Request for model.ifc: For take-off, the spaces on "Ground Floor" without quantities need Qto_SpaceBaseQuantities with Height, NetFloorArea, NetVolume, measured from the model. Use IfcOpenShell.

First a look at what the model holds.

```python
import ifcopenshell
import ifcopenshell.util.element
import ifcopenshell.util.unit

model = ifcopenshell.open("model.ifc")
print(model.schema)
for unit_type in ("LENGTHUNIT", "AREAUNIT", "VOLUMEUNIT"):
    print(unit_type, ifcopenshell.util.unit.calculate_unit_scale(model, unit_type))
storey = next(s for s in model.by_type("IfcBuildingStorey") if s.Name == "Ground Floor")
spaces = [e for e in ifcopenshell.util.element.get_decomposition(storey) if e.is_a("IfcSpace")]
for e in sorted(spaces, key=lambda e: e.id()):
    print(e.id(), e.is_a(), e.Name, list(ifcopenshell.util.element.get_psets(e, qtos_only=True)), sep=" | ")
```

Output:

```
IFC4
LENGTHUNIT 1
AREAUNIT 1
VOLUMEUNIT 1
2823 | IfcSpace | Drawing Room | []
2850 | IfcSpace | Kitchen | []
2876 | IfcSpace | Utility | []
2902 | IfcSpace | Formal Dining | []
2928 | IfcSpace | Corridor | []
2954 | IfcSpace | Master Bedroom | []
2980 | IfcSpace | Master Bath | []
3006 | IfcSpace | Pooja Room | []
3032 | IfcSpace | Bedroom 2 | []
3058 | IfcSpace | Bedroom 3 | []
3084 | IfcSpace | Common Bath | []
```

```python
import ifcopenshell
import ifcopenshell.api.pset
import ifcopenshell.geom
import ifcopenshell.util.element
import ifcopenshell.util.shape
import ifcopenshell.util.unit

model = ifcopenshell.open("model.ifc")
unit_scale = ifcopenshell.util.unit.calculate_unit_scale(model)
area_scale = ifcopenshell.util.unit.calculate_unit_scale(model, "AREAUNIT")
volume_scale = ifcopenshell.util.unit.calculate_unit_scale(model, "VOLUMEUNIT")
settings = ifcopenshell.geom.settings()

storey = next(s for s in model.by_type("IfcBuildingStorey") if s.Name == "Ground Floor")
spaces = [e for e in ifcopenshell.util.element.get_decomposition(storey) if e.is_a("IfcSpace")]

for e in sorted(spaces, key=lambda e: e.id()):
    if ifcopenshell.util.element.get_psets(e, qtos_only=True, should_inherit=False):
        continue
    # Geometry comes back in metres, in the element's own axes.
    shape = ifcopenshell.geom.create_shape(settings, e)
    values = {
        "Height": ifcopenshell.util.shape.get_z(shape.geometry) / unit_scale,
        "NetFloorArea": ifcopenshell.util.shape.get_footprint_area(shape.geometry) / area_scale,
        "NetVolume": ifcopenshell.util.shape.get_volume(shape.geometry) / volume_scale,
    }
    qto = ifcopenshell.api.pset.add_qto(model, product=e, name="Qto_SpaceBaseQuantities")
    ifcopenshell.api.pset.edit_qto(model, qto=qto, properties=values)
    print(e.id(), {k: round(v, 3) for k, v in values.items()})

model.write("model_rev.ifc")
```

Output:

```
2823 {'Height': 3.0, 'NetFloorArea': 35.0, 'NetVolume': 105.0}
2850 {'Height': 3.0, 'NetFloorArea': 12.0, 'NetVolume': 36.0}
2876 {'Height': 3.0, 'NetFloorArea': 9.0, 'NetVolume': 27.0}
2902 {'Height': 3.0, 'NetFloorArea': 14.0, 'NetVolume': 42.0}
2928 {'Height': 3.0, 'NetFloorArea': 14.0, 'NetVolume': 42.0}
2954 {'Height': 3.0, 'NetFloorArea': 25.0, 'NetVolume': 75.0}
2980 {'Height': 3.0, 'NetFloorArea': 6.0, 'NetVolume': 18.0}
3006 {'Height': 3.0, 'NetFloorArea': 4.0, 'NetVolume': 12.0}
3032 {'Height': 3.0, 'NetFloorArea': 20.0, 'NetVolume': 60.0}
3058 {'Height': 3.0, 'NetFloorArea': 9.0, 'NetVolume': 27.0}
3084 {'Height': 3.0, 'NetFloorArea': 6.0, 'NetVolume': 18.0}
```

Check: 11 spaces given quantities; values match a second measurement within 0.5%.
